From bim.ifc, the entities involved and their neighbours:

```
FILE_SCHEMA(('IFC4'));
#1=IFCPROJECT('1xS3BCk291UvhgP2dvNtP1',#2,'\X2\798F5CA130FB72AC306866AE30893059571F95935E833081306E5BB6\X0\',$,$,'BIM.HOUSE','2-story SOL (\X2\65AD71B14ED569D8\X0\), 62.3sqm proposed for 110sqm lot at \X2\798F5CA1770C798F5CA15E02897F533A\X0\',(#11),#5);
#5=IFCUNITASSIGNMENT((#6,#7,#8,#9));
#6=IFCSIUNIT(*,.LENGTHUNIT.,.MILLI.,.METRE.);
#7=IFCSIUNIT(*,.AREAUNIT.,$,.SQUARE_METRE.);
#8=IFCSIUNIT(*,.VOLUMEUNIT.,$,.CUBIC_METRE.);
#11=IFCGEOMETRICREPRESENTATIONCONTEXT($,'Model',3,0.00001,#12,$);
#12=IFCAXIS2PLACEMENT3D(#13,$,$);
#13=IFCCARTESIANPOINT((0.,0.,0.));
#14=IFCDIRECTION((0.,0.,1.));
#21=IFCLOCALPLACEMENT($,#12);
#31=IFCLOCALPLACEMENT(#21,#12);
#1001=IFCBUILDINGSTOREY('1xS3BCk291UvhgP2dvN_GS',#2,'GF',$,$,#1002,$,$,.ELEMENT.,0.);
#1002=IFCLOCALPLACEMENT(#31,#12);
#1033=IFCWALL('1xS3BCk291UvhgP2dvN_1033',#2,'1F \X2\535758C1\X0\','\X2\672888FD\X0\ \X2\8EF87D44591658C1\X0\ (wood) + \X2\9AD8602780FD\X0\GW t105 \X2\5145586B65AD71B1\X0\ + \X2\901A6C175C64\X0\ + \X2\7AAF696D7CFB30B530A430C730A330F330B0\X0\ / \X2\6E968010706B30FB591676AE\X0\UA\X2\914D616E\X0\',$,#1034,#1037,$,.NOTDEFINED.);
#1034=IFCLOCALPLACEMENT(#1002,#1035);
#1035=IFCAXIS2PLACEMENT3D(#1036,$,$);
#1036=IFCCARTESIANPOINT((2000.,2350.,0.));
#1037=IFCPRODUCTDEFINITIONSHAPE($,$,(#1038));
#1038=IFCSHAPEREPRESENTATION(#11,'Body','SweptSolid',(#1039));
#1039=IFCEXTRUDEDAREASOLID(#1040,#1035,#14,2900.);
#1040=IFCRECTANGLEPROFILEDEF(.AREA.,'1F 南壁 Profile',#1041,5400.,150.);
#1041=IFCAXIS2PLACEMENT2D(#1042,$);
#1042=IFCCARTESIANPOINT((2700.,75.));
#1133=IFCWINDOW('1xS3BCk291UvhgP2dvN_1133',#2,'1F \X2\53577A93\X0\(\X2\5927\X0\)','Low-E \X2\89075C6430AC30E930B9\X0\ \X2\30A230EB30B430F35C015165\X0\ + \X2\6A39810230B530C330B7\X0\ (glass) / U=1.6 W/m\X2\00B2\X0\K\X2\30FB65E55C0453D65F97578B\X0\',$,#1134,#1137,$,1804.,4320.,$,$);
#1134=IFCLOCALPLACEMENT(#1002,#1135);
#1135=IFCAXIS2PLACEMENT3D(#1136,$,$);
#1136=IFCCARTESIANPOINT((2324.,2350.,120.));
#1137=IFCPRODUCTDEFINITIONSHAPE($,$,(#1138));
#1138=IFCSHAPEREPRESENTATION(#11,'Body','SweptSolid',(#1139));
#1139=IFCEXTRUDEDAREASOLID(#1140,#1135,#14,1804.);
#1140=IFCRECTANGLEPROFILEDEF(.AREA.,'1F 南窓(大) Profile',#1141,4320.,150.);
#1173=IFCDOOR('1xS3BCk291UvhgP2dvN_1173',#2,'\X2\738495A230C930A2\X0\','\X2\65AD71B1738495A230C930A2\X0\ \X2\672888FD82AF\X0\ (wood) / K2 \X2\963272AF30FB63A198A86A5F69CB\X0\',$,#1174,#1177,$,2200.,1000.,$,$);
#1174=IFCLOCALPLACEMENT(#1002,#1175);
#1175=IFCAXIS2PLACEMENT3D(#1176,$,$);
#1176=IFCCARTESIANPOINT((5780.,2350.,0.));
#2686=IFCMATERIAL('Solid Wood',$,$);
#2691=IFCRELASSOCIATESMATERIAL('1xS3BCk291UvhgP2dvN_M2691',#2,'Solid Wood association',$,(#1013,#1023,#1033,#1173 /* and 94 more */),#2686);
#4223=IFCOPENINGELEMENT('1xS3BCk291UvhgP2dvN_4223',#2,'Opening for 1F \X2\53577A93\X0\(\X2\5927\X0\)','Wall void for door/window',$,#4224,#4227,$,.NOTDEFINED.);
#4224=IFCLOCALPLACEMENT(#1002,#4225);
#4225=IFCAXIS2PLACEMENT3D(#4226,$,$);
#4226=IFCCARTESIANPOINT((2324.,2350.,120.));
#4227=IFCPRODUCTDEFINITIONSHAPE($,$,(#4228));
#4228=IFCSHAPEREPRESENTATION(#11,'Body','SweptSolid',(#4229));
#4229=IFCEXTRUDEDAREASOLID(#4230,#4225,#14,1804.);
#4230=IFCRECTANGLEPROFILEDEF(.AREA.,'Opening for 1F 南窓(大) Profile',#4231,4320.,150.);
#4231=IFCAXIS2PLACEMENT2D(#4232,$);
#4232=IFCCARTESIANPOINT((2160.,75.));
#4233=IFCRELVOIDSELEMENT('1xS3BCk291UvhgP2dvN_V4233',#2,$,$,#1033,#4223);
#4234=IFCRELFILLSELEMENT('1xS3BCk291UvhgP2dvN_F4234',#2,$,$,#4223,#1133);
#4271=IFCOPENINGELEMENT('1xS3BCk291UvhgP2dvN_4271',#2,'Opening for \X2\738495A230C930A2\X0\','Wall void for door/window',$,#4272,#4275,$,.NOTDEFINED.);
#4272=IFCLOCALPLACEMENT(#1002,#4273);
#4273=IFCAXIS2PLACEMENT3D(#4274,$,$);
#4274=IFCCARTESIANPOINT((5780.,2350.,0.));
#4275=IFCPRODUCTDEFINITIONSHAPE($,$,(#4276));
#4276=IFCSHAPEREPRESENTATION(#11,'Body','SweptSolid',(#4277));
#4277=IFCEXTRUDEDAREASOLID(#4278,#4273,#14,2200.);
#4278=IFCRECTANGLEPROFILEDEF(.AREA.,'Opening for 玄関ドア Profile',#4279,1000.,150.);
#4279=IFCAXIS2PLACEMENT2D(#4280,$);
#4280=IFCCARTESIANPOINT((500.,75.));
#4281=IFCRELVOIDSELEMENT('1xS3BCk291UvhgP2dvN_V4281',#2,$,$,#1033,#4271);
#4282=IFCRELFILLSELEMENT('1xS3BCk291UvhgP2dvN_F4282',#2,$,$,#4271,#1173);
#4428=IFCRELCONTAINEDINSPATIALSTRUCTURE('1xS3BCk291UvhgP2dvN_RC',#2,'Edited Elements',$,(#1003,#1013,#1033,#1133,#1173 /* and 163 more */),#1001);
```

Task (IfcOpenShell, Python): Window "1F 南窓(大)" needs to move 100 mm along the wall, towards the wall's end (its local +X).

```python
import ifcopenshell
import ifcopenshell.api.geometry
import ifcopenshell.util.placement
import ifcopenshell.util.unit

model = ifcopenshell.open("bim.ifc")
unit_scale = ifcopenshell.util.unit.calculate_unit_scale(model)

window = model.by_guid("1xS3BCk291UvhgP2dvN_1133")
opening = window.FillsVoids[0].RelatingOpeningElement
wall = opening.VoidsElements[0].RelatingBuildingElement

wall_matrix = ifcopenshell.util.placement.get_local_placement(wall.ObjectPlacement)
shift = wall_matrix[:3, 0] * 0.1 / unit_scale
before = ifcopenshell.util.placement.get_local_placement(window.ObjectPlacement)[:3, 3].copy()

# The window is not placed relative to its opening, so move both.
for product in (opening, window):
    matrix = ifcopenshell.util.placement.get_local_placement(product.ObjectPlacement)
    matrix[:3, 3] += shift
    ifcopenshell.api.geometry.edit_object_placement(model, product=product, matrix=matrix, is_si=False)

after = ifcopenshell.util.placement.get_local_placement(window.ObjectPlacement)[:3, 3]
print("window moved by", (after - before).round(3) + 0.0)

model.write("bim-out.ifc")
```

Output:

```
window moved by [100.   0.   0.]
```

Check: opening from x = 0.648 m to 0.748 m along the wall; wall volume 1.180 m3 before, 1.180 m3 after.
